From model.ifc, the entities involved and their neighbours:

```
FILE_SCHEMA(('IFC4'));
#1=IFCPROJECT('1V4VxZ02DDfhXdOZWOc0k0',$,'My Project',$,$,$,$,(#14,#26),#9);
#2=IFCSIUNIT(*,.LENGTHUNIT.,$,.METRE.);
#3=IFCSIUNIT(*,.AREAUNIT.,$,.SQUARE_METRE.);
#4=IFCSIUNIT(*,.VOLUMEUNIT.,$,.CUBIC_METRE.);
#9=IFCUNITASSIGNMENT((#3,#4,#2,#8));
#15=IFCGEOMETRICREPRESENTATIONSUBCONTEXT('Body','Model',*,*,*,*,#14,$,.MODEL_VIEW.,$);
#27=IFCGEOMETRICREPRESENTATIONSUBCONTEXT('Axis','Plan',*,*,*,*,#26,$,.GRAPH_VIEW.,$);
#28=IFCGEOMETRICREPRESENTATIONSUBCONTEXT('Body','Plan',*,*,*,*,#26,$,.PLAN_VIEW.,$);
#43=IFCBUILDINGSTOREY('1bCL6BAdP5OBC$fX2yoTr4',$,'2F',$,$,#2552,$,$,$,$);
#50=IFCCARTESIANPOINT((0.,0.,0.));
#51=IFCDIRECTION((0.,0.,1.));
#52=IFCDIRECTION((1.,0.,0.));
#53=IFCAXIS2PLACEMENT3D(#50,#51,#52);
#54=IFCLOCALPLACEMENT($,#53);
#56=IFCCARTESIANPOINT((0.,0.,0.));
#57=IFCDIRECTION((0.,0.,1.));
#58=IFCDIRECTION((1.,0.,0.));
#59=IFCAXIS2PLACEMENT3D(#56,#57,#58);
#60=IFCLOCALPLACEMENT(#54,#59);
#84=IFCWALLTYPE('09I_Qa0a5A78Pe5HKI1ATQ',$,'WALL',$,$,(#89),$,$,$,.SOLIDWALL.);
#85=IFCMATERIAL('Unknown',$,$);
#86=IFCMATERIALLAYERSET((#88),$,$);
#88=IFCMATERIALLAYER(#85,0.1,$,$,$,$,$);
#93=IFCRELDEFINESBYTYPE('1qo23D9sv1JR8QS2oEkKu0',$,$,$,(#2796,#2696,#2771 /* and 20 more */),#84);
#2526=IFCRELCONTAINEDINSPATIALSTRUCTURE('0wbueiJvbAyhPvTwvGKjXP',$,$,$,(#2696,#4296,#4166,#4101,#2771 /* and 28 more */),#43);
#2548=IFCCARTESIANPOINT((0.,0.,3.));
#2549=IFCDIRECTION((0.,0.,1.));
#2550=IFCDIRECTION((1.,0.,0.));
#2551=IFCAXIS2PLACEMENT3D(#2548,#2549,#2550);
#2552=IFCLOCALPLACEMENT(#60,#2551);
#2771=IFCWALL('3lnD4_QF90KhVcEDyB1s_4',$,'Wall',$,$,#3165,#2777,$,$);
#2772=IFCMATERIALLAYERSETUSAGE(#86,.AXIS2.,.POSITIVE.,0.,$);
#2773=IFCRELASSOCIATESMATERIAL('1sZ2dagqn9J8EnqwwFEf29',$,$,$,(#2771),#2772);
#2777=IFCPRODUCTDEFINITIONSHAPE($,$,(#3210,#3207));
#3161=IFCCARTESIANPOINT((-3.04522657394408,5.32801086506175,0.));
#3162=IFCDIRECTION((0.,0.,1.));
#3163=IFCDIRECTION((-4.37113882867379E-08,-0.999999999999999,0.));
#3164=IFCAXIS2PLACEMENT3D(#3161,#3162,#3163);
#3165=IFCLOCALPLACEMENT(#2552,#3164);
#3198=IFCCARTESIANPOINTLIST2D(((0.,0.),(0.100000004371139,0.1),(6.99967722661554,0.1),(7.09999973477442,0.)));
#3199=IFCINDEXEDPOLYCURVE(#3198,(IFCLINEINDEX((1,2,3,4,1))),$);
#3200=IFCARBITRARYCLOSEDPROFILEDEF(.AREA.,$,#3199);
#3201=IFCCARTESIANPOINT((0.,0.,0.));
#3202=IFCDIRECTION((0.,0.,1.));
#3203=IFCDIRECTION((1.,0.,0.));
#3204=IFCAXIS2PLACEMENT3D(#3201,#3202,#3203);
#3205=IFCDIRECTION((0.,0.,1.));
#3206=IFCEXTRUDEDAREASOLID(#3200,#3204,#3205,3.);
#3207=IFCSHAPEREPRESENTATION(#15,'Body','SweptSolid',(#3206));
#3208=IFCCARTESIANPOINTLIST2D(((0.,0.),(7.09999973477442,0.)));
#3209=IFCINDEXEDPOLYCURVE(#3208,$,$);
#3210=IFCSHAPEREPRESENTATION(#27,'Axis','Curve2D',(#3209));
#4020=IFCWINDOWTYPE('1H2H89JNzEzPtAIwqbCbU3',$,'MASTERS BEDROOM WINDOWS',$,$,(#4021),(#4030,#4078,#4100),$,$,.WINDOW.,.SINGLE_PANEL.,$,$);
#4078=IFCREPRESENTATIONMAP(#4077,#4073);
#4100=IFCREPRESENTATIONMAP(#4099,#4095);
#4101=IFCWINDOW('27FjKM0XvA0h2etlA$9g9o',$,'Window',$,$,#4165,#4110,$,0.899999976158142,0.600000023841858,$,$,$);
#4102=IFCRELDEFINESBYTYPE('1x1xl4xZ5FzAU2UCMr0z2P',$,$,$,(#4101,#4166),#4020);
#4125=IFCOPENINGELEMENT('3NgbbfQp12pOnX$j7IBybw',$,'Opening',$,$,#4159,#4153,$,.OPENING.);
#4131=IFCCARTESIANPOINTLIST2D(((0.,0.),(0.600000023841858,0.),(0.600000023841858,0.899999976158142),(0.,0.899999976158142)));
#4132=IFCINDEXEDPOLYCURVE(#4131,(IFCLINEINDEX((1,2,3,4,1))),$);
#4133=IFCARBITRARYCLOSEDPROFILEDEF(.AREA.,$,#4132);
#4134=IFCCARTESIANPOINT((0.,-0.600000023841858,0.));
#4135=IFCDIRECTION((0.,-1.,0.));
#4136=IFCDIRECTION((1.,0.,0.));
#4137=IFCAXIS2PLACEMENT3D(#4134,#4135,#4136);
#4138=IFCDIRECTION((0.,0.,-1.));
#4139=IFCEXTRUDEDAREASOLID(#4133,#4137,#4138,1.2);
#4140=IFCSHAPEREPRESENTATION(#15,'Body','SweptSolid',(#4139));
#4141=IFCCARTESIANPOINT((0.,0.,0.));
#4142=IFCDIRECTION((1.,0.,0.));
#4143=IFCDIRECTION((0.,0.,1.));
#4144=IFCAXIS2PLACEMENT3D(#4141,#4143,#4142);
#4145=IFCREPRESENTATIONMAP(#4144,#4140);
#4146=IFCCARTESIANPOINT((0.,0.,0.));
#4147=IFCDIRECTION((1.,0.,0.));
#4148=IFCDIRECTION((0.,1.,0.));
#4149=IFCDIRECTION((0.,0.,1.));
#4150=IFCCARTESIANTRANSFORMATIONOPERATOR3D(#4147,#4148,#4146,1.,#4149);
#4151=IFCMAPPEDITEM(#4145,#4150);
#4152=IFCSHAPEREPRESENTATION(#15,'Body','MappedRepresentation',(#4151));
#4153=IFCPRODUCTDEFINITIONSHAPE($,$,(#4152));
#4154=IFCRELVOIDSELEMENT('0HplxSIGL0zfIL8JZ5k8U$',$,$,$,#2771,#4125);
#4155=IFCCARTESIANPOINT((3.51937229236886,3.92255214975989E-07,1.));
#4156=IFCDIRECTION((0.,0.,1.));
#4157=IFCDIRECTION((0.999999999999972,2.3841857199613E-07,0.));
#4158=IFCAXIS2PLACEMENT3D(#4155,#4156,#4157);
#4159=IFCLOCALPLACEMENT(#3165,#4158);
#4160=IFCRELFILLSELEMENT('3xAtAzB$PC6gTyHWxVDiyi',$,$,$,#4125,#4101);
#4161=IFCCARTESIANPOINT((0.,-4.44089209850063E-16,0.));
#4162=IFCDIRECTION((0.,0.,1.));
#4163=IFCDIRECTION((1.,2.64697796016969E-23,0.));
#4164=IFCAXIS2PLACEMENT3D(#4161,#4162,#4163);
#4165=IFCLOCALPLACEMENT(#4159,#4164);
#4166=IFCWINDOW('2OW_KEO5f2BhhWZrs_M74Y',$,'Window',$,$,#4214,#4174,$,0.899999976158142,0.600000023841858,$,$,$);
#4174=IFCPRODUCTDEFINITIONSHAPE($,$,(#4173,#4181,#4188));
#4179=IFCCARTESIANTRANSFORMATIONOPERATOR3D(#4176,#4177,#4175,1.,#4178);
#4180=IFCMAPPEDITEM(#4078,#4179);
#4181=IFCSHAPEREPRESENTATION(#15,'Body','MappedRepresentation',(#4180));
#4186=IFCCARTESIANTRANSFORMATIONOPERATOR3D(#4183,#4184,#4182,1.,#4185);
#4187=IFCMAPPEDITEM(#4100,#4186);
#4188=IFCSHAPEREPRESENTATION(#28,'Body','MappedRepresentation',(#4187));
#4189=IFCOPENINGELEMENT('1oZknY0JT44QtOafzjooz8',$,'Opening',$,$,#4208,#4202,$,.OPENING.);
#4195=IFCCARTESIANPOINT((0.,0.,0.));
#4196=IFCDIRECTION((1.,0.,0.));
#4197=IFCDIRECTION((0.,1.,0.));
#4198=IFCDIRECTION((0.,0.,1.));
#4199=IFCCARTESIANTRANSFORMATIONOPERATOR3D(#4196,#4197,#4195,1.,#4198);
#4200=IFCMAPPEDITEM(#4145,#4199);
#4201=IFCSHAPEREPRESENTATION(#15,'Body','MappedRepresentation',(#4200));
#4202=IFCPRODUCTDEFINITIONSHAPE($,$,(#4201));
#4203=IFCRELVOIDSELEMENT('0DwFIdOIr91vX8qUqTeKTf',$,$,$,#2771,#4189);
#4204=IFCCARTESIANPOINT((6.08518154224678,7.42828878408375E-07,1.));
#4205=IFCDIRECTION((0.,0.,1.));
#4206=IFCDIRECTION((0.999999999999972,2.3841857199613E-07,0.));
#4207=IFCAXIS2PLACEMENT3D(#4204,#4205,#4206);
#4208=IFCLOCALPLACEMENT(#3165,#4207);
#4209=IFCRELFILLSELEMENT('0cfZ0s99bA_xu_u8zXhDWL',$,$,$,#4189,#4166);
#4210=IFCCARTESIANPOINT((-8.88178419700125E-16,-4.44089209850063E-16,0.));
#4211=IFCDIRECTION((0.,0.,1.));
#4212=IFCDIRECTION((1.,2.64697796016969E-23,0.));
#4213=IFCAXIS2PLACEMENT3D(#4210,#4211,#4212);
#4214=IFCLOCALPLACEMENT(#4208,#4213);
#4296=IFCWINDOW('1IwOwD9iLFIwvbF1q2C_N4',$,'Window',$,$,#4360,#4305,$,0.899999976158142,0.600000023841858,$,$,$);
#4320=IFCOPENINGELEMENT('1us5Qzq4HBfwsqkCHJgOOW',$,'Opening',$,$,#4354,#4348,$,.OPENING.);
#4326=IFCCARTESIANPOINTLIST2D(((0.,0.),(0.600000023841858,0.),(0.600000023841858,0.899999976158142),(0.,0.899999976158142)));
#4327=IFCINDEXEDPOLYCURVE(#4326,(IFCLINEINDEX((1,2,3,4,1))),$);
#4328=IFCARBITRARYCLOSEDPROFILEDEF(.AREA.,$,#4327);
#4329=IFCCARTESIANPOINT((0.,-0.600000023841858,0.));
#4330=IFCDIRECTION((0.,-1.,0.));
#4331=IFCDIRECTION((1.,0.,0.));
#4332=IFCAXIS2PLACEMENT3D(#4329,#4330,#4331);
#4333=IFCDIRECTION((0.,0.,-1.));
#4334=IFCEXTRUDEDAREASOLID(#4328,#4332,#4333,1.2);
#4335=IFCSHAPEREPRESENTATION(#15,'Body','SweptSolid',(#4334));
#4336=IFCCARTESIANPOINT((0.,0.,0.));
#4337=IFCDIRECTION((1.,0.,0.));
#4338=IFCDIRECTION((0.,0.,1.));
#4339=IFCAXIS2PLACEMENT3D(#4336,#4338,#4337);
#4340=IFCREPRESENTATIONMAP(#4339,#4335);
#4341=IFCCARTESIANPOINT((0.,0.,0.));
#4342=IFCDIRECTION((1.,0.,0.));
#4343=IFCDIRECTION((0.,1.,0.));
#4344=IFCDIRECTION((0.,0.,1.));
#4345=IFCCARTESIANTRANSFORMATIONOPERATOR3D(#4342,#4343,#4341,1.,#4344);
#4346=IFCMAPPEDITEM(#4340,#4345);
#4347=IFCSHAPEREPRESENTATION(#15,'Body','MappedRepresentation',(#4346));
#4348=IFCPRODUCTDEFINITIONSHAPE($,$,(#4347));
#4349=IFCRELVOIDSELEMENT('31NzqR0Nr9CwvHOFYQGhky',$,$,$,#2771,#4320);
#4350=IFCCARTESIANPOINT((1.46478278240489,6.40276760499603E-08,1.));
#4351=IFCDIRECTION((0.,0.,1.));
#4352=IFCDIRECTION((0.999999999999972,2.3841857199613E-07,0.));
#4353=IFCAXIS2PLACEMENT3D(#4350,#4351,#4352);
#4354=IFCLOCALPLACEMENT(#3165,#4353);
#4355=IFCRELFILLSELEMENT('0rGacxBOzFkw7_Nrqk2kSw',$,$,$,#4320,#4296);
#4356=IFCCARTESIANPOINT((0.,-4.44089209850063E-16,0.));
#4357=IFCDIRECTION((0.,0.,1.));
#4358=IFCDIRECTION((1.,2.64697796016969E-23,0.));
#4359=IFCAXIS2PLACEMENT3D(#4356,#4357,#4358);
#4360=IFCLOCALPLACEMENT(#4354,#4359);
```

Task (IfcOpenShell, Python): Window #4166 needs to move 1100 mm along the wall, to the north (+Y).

```python
import ifcopenshell
import ifcopenshell.api.geometry
import ifcopenshell.util.placement

model = ifcopenshell.open("model.ifc")

window = model.by_guid("2OW_KEO5f2BhhWZrs_M74Y")
opening = window.FillsVoids[0].RelatingOpeningElement
wall = opening.VoidsElements[0].RelatingBuildingElement

wall_matrix = ifcopenshell.util.placement.get_local_placement(wall.ObjectPlacement)
shift = wall_matrix[:3, 0] * -1.1
before = ifcopenshell.util.placement.get_local_placement(window.ObjectPlacement)[:3, 3].copy()

# The window is placed relative to its opening, so it follows when the opening moves.
matrix = ifcopenshell.util.placement.get_local_placement(opening.ObjectPlacement)
matrix[:3, 3] += shift
ifcopenshell.api.geometry.edit_object_placement(
    model, product=opening, matrix=matrix, is_si=False, should_transform_children=True
)

after = ifcopenshell.util.placement.get_local_placement(window.ObjectPlacement)[:3, 3]
print("window moved by", (after - before).round(3) + 0.0)

model.write("model_v2.ifc")
```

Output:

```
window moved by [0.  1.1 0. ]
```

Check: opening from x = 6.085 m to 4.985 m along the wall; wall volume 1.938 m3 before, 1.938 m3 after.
